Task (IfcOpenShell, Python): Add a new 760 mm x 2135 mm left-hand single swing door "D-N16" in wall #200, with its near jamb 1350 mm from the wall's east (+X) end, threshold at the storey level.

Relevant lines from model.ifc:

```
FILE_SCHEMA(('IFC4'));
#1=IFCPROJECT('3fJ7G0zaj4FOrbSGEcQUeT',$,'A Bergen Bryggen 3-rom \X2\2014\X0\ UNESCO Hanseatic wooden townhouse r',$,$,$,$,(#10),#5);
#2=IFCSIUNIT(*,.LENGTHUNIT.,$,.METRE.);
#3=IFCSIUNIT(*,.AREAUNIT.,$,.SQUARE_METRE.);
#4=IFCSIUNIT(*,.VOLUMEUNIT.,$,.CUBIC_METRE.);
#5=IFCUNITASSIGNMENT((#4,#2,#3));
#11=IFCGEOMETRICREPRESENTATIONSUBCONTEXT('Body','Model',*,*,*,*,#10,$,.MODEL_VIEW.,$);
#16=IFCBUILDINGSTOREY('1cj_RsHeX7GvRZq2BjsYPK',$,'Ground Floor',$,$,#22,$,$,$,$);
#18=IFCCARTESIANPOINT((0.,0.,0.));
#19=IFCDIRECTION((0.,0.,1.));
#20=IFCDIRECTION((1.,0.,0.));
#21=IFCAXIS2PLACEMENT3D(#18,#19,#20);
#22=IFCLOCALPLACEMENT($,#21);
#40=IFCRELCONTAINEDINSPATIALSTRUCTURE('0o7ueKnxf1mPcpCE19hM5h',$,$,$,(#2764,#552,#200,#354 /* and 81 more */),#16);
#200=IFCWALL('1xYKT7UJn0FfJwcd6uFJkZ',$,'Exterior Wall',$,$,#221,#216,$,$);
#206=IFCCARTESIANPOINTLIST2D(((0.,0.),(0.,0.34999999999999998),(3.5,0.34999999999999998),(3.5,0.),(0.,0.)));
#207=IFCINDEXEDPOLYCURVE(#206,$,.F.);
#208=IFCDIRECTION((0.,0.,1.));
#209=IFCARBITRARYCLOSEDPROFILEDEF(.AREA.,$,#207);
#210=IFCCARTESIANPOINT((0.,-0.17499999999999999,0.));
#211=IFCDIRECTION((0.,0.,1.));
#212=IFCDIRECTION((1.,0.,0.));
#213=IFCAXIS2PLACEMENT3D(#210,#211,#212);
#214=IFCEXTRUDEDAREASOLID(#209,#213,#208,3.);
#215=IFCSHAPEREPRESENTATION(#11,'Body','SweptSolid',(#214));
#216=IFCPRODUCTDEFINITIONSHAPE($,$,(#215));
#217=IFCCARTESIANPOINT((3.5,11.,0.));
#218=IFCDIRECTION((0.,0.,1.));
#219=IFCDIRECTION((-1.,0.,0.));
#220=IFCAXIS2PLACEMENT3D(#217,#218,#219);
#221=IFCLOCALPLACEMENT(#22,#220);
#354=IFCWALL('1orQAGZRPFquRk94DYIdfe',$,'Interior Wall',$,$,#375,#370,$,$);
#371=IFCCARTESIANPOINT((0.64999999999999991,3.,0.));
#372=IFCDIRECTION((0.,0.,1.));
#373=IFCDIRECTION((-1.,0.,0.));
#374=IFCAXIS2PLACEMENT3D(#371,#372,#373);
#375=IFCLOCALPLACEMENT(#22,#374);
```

```python
import numpy as np
import ifcopenshell
import ifcopenshell.api.feature
import ifcopenshell.api.geometry
import ifcopenshell.api.root
import ifcopenshell.api.spatial
import ifcopenshell.geom
import ifcopenshell.util.element
import ifcopenshell.util.placement
import ifcopenshell.util.representation
import ifcopenshell.util.shape
import ifcopenshell.util.unit

model = ifcopenshell.open("model.ifc")
unit_scale = ifcopenshell.util.unit.calculate_unit_scale(model)
settings = ifcopenshell.geom.settings()


def volume(element):
    """Net volume in cubic metres, openings subtracted."""
    shape = ifcopenshell.geom.create_shape(settings, element)
    return ifcopenshell.util.shape.get_volume(shape.geometry)


wall = model.by_guid("1xYKT7UJn0FfJwcd6uFJkZ")
storey = ifcopenshell.util.element.get_container(wall, ifc_class="IfcBuildingStorey")
context = ifcopenshell.util.representation.get_context(model, "Model", "Body", "MODEL_VIEW")
before = volume(wall)

width, height, from_end, sill = 0.76, 2.135, 1.35, 0.0  # metres

# The wall runs along its own X axis, and the end named is its -X end.
wall_shape = ifcopenshell.geom.create_shape(settings, wall)
x, y, z = ifcopenshell.util.shape.get_vertices(wall_shape.geometry).T
start = x.min() + from_end
face, thickness = float(y.min()), float(y.max() - y.min())
wall_matrix = ifcopenshell.util.placement.get_local_placement(wall.ObjectPlacement)
level = ifcopenshell.util.placement.get_local_placement(storey.ObjectPlacement)[2, 3]


def in_wall(x, y):
    """Placement at x, y metres in the wall's axes, at sill height."""
    matrix = wall_matrix.copy()
    matrix[:, 3] = wall_matrix @ np.array([x / unit_scale, y / unit_scale, 0.0, 1.0])
    matrix[2, 3] = level + sill / unit_scale
    return matrix


# Opening: a box that overshoots both wall faces by 50 mm.
opening = ifcopenshell.api.root.create_entity(model, ifc_class="IfcOpeningElement", predefined_type="OPENING")
box = ifcopenshell.api.geometry.add_wall_representation(
    model, context=context, length=width, height=height, thickness=thickness + 0.1
)
ifcopenshell.api.geometry.assign_representation(model, product=opening, representation=box)
ifcopenshell.api.geometry.edit_object_placement(model, product=opening, matrix=in_wall(start, face - 0.05), is_si=False)
ifcopenshell.api.feature.add_feature(model, feature=opening, element=wall)

door = ifcopenshell.api.root.create_entity(model, ifc_class="IfcDoor", name="D-N16", predefined_type="DOOR")
door.OverallWidth, door.OverallHeight = width / unit_scale, height / unit_scale
door.OperationType = "SINGLE_SWING_LEFT"
body = ifcopenshell.api.geometry.add_door_representation(
    model,
    context=context,
    overall_width=door.OverallWidth,
    overall_height=door.OverallHeight,
    operation_type="SINGLE_SWING_LEFT",
    lining_properties={"LiningDepth": thickness / unit_scale, "ThresholdDepth": thickness / unit_scale},
)
ifcopenshell.api.geometry.assign_representation(model, product=door, representation=body)
ifcopenshell.api.spatial.assign_container(model, products=[door], relating_structure=storey)
ifcopenshell.api.feature.add_filling(model, opening=opening, element=door)

# The lining spans the wall, so the door starts at the wall face.
ifcopenshell.api.geometry.edit_object_placement(model, product=door, matrix=in_wall(start, face), is_si=False)

after = volume(wall)

print(f"wall volume {before:.3f} -> {after:.3f} m3")

model.write("model_v2.ifc")
```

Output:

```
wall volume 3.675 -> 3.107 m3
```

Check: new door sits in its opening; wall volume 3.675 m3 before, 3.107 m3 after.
